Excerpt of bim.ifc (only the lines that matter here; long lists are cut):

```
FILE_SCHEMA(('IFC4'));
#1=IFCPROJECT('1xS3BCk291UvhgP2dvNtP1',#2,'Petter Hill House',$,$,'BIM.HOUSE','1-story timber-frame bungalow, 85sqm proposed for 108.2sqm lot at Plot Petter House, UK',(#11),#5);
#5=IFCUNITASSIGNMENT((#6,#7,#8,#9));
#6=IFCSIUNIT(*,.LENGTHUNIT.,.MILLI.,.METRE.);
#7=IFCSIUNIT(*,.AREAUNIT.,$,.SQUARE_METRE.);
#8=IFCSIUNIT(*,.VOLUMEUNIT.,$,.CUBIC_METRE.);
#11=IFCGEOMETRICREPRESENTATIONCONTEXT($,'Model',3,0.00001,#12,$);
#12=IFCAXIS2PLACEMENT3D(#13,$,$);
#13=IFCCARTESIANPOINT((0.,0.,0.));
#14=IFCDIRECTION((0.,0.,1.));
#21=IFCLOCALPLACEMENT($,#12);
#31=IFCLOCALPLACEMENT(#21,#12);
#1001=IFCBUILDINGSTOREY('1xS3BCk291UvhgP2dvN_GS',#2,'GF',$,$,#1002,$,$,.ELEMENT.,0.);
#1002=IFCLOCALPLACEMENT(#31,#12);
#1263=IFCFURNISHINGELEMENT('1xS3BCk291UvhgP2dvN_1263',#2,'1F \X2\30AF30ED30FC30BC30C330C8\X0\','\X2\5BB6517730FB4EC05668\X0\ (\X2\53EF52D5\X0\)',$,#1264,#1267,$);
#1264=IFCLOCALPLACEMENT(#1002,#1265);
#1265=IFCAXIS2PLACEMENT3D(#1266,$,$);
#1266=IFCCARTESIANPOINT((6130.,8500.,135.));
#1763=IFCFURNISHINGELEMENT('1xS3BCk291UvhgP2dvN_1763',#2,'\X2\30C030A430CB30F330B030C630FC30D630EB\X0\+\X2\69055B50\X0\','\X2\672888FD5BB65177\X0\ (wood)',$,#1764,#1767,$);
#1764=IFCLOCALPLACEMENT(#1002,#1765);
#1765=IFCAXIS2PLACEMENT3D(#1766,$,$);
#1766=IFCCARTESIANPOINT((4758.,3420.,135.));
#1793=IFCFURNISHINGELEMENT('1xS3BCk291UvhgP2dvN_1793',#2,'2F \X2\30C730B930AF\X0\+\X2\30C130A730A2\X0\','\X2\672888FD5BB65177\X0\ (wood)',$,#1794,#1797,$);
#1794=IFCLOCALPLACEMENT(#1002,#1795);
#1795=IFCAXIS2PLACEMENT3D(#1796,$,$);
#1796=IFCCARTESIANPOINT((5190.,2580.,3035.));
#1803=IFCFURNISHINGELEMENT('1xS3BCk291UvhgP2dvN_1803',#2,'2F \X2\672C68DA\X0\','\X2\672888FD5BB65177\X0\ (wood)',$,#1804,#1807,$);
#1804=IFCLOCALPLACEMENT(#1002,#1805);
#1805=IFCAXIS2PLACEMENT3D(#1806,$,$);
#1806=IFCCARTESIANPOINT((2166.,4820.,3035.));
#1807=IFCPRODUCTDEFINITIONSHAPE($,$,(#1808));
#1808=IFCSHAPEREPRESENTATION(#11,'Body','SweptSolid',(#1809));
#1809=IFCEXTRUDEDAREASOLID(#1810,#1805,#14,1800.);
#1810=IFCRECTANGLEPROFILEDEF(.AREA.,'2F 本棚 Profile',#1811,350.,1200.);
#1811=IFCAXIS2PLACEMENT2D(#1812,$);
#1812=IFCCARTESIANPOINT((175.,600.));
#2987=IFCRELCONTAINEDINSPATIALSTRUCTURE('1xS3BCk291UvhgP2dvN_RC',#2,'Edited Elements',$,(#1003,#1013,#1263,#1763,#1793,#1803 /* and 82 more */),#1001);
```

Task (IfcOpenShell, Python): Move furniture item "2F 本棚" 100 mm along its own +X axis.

```python
import ifcopenshell
import ifcopenshell.api.geometry
import ifcopenshell.util.placement

model = ifcopenshell.open("bim.ifc")

item = model.by_id(1803)
matrix = ifcopenshell.util.placement.get_local_placement(item.ObjectPlacement)
matrix[:3, 3] += matrix[:3, 0] * 100.0
ifcopenshell.api.geometry.edit_object_placement(model, product=item, matrix=matrix, is_si=False)

print(ifcopenshell.util.placement.get_local_placement(item.ObjectPlacement).round(3) + 0.0)

model.write("bim_v2.ifc")
```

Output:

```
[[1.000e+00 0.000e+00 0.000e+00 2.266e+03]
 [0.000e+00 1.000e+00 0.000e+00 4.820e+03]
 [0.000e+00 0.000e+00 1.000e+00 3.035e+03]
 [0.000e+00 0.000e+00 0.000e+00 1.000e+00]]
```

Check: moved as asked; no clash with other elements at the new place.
